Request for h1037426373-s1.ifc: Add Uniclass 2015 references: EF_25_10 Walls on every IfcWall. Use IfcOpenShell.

First a look at what the model holds.

```python
import ifcopenshell

model = ifcopenshell.open("h1037426373-s1.ifc")
print(model.schema)
print("classifications:", [c.Name for c in model.by_type("IfcClassification")])
for ifc_class in ("IfcDoor", "IfcRoof", "IfcStair", "IfcWall", "IfcWindow"):
    print(ifc_class, len(model.by_type(ifc_class)))
```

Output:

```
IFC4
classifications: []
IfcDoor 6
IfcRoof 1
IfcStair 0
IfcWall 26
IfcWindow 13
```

```python
import ifcopenshell
import ifcopenshell.api.classification

model = ifcopenshell.open("h1037426373-s1.ifc")

system = ifcopenshell.api.classification.add_classification(model, classification="Uniclass 2015")

codes = {
    "IfcWall": ("EF_25_10", "Walls"),
}
for ifc_class, (code, name) in codes.items():
    products = model.by_type(ifc_class)
    ifcopenshell.api.classification.add_reference(
        model, products=products, classification=system, identification=code, name=name
    )
    print(code, len(products))

model.write("h1037426373-s1_v2.ifc")
```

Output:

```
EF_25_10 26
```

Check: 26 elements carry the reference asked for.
